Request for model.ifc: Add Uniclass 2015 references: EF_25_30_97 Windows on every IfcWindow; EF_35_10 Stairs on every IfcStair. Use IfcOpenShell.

First a look at what the model holds.

```python
import ifcopenshell

model = ifcopenshell.open("model.ifc")
print(model.schema)
print("classifications:", [c.Name for c in model.by_type("IfcClassification")])
for ifc_class in ("IfcDoor", "IfcRoof", "IfcStair", "IfcWall", "IfcWindow"):
    print(ifc_class, len(model.by_type(ifc_class)))
```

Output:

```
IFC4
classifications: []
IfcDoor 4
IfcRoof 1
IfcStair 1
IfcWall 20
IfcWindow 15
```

```python
import ifcopenshell
import ifcopenshell.api.classification

model = ifcopenshell.open("model.ifc")

system = ifcopenshell.api.classification.add_classification(model, classification="Uniclass 2015")

codes = {
    "IfcWindow": ("EF_25_30_97", "Windows"),
    "IfcStair": ("EF_35_10", "Stairs"),
}
for ifc_class, (code, name) in codes.items():
    products = model.by_type(ifc_class)
    ifcopenshell.api.classification.add_reference(
        model, products=products, classification=system, identification=code, name=name
    )
    print(code, len(products))

model.write("model-out.ifc")
```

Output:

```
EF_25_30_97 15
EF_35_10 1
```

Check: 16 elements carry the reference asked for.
